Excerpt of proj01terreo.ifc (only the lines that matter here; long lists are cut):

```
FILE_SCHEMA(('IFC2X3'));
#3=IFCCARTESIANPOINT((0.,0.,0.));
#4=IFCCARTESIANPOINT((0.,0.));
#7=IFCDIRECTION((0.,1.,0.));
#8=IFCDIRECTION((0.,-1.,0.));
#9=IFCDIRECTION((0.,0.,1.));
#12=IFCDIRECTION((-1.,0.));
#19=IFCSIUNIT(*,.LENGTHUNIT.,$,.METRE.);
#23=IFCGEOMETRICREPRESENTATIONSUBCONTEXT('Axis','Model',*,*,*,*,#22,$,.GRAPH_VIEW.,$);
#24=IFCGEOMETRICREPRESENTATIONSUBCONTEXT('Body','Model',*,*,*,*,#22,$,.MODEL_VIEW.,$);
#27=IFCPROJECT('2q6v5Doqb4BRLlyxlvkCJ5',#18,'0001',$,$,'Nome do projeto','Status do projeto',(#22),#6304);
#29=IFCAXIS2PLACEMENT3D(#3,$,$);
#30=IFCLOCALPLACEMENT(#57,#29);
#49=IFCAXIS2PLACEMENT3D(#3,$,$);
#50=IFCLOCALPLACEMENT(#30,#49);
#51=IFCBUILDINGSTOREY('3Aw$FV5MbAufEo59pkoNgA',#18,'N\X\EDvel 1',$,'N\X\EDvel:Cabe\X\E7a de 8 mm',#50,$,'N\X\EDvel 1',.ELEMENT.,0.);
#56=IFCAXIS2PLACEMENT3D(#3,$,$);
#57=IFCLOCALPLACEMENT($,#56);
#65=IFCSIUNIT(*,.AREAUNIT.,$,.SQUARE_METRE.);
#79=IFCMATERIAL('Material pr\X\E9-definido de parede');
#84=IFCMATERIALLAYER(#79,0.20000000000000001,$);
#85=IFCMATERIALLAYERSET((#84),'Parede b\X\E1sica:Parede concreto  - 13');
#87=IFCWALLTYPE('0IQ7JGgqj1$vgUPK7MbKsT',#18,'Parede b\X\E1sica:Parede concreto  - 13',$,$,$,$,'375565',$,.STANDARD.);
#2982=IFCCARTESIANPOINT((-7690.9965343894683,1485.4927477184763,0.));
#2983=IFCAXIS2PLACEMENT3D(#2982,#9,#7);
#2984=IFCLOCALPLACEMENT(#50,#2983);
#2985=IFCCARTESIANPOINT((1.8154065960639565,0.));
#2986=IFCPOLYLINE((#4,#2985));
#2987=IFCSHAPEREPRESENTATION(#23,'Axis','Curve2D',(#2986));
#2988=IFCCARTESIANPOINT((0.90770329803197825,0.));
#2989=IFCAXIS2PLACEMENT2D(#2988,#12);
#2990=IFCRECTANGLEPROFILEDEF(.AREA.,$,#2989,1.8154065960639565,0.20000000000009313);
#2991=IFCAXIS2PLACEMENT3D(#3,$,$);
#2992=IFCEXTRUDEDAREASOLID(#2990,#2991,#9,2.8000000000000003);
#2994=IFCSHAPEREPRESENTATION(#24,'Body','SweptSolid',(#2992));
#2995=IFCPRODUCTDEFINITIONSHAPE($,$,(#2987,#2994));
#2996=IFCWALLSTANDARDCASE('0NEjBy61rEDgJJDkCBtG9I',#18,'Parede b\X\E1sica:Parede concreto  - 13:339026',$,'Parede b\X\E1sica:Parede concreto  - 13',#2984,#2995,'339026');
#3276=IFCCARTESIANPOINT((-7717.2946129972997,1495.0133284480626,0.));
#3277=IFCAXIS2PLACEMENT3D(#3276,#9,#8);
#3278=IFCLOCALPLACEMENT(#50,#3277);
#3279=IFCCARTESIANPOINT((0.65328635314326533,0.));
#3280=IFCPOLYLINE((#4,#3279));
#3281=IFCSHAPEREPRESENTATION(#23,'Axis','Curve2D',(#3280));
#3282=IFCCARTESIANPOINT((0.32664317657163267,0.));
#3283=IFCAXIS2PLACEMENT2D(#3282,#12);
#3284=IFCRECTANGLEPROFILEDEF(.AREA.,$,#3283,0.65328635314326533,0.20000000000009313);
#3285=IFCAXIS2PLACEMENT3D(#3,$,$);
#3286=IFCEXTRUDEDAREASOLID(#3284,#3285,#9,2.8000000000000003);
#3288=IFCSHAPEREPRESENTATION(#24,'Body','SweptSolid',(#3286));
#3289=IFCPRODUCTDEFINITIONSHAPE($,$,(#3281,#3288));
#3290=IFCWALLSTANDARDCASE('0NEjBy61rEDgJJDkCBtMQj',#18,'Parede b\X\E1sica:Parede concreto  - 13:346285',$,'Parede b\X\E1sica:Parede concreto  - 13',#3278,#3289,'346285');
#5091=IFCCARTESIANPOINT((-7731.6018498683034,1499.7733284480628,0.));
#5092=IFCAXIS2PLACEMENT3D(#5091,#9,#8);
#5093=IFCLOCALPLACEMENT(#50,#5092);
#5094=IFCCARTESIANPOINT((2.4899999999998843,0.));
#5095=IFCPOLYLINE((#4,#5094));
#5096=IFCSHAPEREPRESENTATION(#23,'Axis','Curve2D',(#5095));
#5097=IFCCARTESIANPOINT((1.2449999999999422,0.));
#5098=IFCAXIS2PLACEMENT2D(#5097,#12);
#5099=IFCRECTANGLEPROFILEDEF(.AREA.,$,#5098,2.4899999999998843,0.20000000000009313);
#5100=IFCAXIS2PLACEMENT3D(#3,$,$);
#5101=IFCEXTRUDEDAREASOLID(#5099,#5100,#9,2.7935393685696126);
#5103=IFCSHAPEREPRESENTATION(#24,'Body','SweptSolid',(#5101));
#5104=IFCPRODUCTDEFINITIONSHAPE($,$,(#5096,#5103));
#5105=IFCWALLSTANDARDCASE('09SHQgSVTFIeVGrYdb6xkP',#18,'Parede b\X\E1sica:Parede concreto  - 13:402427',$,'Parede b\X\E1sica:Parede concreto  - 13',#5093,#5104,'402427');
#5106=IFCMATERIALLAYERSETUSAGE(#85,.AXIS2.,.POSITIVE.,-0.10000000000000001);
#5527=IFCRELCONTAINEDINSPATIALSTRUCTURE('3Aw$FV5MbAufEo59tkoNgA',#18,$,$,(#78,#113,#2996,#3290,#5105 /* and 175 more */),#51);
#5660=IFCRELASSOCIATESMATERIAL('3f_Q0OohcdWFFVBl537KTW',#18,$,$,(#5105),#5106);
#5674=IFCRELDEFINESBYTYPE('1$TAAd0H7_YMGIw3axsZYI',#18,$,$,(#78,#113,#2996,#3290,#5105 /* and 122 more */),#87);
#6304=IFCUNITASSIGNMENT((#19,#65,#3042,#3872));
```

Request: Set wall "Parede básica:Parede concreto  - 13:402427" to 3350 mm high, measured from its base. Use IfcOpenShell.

```python
import ifcopenshell
import ifcopenshell.geom
import ifcopenshell.util.representation
import ifcopenshell.util.shape
import ifcopenshell.util.unit

model = ifcopenshell.open("proj01terreo.ifc")
unit_scale = ifcopenshell.util.unit.calculate_unit_scale(model)
settings = ifcopenshell.geom.settings()


def volume(element):
    """Net volume in cubic metres, openings subtracted."""
    shape = ifcopenshell.geom.create_shape(settings, element)
    return ifcopenshell.util.shape.get_volume(shape.geometry)


wall = model.by_id(5105)
before = volume(wall)

body = ifcopenshell.util.representation.get_representation(wall, "Model", "Body")
solid = body.Items[0]
old_height = solid.Depth
solid.Depth = 3.35 / unit_scale
after = volume(wall)

print(f"height {old_height:g} -> {solid.Depth:g}, volume {before:.3f} -> {after:.3f} m3")

model.write("proj01terreo_v2.ifc")
```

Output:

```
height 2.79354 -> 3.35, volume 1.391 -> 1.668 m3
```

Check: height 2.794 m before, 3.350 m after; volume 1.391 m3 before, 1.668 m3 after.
